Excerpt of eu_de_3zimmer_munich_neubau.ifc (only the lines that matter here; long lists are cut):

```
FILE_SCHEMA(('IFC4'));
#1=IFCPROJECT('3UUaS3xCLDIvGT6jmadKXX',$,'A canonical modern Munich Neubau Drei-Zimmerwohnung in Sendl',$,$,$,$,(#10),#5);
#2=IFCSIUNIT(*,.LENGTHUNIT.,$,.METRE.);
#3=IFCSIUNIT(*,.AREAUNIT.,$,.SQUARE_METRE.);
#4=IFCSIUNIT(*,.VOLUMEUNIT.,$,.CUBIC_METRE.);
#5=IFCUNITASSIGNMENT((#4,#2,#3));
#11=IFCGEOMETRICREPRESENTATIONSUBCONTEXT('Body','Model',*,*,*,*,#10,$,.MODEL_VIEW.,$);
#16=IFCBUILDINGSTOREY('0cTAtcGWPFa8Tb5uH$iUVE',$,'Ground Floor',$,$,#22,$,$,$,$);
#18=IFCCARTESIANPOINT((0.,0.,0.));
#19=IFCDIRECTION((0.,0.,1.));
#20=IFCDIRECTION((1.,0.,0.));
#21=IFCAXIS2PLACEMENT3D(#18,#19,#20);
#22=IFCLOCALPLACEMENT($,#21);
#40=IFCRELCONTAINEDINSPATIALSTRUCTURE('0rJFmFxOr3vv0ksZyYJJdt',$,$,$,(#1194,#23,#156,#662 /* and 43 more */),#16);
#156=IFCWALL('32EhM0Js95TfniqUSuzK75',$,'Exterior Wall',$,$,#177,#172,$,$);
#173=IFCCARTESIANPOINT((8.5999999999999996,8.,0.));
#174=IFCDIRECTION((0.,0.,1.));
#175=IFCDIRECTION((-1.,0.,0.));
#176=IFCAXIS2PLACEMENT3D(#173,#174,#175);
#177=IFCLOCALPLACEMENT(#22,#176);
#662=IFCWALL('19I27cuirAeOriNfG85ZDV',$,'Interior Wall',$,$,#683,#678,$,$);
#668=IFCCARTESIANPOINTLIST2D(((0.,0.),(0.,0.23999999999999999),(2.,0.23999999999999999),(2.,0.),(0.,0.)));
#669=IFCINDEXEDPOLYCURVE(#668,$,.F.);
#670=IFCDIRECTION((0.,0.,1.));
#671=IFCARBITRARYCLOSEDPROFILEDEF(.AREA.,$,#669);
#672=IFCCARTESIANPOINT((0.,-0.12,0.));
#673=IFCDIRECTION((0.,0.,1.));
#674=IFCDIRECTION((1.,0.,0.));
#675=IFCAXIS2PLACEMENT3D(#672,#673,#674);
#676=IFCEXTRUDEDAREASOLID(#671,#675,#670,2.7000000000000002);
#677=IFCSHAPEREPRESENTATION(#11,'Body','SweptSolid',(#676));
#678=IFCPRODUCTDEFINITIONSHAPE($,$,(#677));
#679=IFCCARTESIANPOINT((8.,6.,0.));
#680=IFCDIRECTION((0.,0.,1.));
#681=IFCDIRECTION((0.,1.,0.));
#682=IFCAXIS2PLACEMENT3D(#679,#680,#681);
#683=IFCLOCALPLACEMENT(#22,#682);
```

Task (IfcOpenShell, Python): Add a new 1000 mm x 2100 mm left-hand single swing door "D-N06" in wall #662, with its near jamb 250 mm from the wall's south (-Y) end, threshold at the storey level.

```python
import numpy as np
import ifcopenshell
import ifcopenshell.api.feature
import ifcopenshell.api.geometry
import ifcopenshell.api.root
import ifcopenshell.api.spatial
import ifcopenshell.geom
import ifcopenshell.util.element
import ifcopenshell.util.placement
import ifcopenshell.util.representation
import ifcopenshell.util.shape
import ifcopenshell.util.unit

model = ifcopenshell.open("eu_de_3zimmer_munich_neubau.ifc")
unit_scale = ifcopenshell.util.unit.calculate_unit_scale(model)
settings = ifcopenshell.geom.settings()


def volume(element):
    """Net volume in cubic metres, openings subtracted."""
    shape = ifcopenshell.geom.create_shape(settings, element)
    return ifcopenshell.util.shape.get_volume(shape.geometry)


wall = model.by_id(662)
storey = ifcopenshell.util.element.get_container(wall, ifc_class="IfcBuildingStorey")
context = ifcopenshell.util.representation.get_context(model, "Model", "Body", "MODEL_VIEW")
before = volume(wall)

width, height, from_end, sill = 1, 2.1, 0.25, 0.0  # metres

# The wall runs along its own X axis, and the end named is its -X end.
wall_shape = ifcopenshell.geom.create_shape(settings, wall)
x, y, z = ifcopenshell.util.shape.get_vertices(wall_shape.geometry).T
start = x.min() + from_end
face, thickness = float(y.min()), float(y.max() - y.min())
wall_matrix = ifcopenshell.util.placement.get_local_placement(wall.ObjectPlacement)
level = ifcopenshell.util.placement.get_local_placement(storey.ObjectPlacement)[2, 3]


def in_wall(x, y):
    """Placement at x, y metres in the wall's axes, at sill height."""
    matrix = wall_matrix.copy()
    matrix[:, 3] = wall_matrix @ np.array([x / unit_scale, y / unit_scale, 0.0, 1.0])
    matrix[2, 3] = level + sill / unit_scale
    return matrix


# Opening: a box that overshoots both wall faces by 50 mm.
opening = ifcopenshell.api.root.create_entity(model, ifc_class="IfcOpeningElement", predefined_type="OPENING")
box = ifcopenshell.api.geometry.add_wall_representation(
    model, context=context, length=width, height=height, thickness=thickness + 0.1
)
ifcopenshell.api.geometry.assign_representation(model, product=opening, representation=box)
ifcopenshell.api.geometry.edit_object_placement(model, product=opening, matrix=in_wall(start, face - 0.05), is_si=False)
ifcopenshell.api.feature.add_feature(model, feature=opening, element=wall)

door = ifcopenshell.api.root.create_entity(model, ifc_class="IfcDoor", name="D-N06", predefined_type="DOOR")
door.OverallWidth, door.OverallHeight = width / unit_scale, height / unit_scale
door.OperationType = "SINGLE_SWING_LEFT"
body = ifcopenshell.api.geometry.add_door_representation(
    model,
    context=context,
    overall_width=door.OverallWidth,
    overall_height=door.OverallHeight,
    operation_type="SINGLE_SWING_LEFT",
    lining_properties={"LiningDepth": thickness / unit_scale, "ThresholdDepth": thickness / unit_scale},
)
ifcopenshell.api.geometry.assign_representation(model, product=door, representation=body)
ifcopenshell.api.spatial.assign_container(model, products=[door], relating_structure=storey)
ifcopenshell.api.feature.add_filling(model, opening=opening, element=door)

# The lining spans the wall, so the door starts at the wall face.
ifcopenshell.api.geometry.edit_object_placement(model, product=door, matrix=in_wall(start, face), is_si=False)

after = volume(wall)

print(f"wall volume {before:.3f} -> {after:.3f} m3")

model.write("eu_de_3zimmer_munich_neubau_rev.ifc")
```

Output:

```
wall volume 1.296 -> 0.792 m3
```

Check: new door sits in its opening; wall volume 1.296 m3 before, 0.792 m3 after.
